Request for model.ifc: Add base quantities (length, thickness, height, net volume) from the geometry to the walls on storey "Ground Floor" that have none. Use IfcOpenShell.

First a look at what the model holds.

```python
import ifcopenshell
import ifcopenshell.util.element
import ifcopenshell.util.unit

model = ifcopenshell.open("model.ifc")
print(model.schema)
for unit_type in ("LENGTHUNIT", "AREAUNIT", "VOLUMEUNIT"):
    print(unit_type, ifcopenshell.util.unit.calculate_unit_scale(model, unit_type))
storey = next(s for s in model.by_type("IfcBuildingStorey") if s.Name == "Ground Floor")
walls = [e for e in ifcopenshell.util.element.get_decomposition(storey) if e.is_a("IfcWall")]
for e in sorted(walls, key=lambda e: e.id()):
    print(e.id(), e.is_a(), e.Name, list(ifcopenshell.util.element.get_psets(e, qtos_only=True)), sep=" | ")
```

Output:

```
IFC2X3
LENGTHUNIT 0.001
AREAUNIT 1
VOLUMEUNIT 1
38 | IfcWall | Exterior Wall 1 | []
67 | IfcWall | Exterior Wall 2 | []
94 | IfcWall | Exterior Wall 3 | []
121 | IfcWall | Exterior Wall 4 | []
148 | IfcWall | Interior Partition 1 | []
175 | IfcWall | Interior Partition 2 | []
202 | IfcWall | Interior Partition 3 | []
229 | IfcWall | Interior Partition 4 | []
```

```python
import ifcopenshell
import ifcopenshell.api.pset
import ifcopenshell.geom
import ifcopenshell.util.element
import ifcopenshell.util.shape
import ifcopenshell.util.unit

model = ifcopenshell.open("model.ifc")
unit_scale = ifcopenshell.util.unit.calculate_unit_scale(model)
volume_scale = ifcopenshell.util.unit.calculate_unit_scale(model, "VOLUMEUNIT")
settings = ifcopenshell.geom.settings()

storey = next(s for s in model.by_type("IfcBuildingStorey") if s.Name == "Ground Floor")
walls = [e for e in ifcopenshell.util.element.get_decomposition(storey) if e.is_a("IfcWall")]

for e in sorted(walls, key=lambda e: e.id()):
    if ifcopenshell.util.element.get_psets(e, qtos_only=True, should_inherit=False):
        continue
    # Geometry comes back in metres, in the element's own axes.
    shape = ifcopenshell.geom.create_shape(settings, e)
    values = {
        "Length": ifcopenshell.util.shape.get_x(shape.geometry) / unit_scale,
        "Width": ifcopenshell.util.shape.get_y(shape.geometry) / unit_scale,
        "Height": ifcopenshell.util.shape.get_z(shape.geometry) / unit_scale,
        "NetVolume": ifcopenshell.util.shape.get_volume(shape.geometry) / volume_scale,
    }
    qto = ifcopenshell.api.pset.add_qto(model, product=e, name="BaseQuantities")
    ifcopenshell.api.pset.edit_qto(model, qto=qto, properties=values)
    print(e.id(), {k: round(v, 3) for k, v in values.items()})

model.write("model_edited.ifc")
```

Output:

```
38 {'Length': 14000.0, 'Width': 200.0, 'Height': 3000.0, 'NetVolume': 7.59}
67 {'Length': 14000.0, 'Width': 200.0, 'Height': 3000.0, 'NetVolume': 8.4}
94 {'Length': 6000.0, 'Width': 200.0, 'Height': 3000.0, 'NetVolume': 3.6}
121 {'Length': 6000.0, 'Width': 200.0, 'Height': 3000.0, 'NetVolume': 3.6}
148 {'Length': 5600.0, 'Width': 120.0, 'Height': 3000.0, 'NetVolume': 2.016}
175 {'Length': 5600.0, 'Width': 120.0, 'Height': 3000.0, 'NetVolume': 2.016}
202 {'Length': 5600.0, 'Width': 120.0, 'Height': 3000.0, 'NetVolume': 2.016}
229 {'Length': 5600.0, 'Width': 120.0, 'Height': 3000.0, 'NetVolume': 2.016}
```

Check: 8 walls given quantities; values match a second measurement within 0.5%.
